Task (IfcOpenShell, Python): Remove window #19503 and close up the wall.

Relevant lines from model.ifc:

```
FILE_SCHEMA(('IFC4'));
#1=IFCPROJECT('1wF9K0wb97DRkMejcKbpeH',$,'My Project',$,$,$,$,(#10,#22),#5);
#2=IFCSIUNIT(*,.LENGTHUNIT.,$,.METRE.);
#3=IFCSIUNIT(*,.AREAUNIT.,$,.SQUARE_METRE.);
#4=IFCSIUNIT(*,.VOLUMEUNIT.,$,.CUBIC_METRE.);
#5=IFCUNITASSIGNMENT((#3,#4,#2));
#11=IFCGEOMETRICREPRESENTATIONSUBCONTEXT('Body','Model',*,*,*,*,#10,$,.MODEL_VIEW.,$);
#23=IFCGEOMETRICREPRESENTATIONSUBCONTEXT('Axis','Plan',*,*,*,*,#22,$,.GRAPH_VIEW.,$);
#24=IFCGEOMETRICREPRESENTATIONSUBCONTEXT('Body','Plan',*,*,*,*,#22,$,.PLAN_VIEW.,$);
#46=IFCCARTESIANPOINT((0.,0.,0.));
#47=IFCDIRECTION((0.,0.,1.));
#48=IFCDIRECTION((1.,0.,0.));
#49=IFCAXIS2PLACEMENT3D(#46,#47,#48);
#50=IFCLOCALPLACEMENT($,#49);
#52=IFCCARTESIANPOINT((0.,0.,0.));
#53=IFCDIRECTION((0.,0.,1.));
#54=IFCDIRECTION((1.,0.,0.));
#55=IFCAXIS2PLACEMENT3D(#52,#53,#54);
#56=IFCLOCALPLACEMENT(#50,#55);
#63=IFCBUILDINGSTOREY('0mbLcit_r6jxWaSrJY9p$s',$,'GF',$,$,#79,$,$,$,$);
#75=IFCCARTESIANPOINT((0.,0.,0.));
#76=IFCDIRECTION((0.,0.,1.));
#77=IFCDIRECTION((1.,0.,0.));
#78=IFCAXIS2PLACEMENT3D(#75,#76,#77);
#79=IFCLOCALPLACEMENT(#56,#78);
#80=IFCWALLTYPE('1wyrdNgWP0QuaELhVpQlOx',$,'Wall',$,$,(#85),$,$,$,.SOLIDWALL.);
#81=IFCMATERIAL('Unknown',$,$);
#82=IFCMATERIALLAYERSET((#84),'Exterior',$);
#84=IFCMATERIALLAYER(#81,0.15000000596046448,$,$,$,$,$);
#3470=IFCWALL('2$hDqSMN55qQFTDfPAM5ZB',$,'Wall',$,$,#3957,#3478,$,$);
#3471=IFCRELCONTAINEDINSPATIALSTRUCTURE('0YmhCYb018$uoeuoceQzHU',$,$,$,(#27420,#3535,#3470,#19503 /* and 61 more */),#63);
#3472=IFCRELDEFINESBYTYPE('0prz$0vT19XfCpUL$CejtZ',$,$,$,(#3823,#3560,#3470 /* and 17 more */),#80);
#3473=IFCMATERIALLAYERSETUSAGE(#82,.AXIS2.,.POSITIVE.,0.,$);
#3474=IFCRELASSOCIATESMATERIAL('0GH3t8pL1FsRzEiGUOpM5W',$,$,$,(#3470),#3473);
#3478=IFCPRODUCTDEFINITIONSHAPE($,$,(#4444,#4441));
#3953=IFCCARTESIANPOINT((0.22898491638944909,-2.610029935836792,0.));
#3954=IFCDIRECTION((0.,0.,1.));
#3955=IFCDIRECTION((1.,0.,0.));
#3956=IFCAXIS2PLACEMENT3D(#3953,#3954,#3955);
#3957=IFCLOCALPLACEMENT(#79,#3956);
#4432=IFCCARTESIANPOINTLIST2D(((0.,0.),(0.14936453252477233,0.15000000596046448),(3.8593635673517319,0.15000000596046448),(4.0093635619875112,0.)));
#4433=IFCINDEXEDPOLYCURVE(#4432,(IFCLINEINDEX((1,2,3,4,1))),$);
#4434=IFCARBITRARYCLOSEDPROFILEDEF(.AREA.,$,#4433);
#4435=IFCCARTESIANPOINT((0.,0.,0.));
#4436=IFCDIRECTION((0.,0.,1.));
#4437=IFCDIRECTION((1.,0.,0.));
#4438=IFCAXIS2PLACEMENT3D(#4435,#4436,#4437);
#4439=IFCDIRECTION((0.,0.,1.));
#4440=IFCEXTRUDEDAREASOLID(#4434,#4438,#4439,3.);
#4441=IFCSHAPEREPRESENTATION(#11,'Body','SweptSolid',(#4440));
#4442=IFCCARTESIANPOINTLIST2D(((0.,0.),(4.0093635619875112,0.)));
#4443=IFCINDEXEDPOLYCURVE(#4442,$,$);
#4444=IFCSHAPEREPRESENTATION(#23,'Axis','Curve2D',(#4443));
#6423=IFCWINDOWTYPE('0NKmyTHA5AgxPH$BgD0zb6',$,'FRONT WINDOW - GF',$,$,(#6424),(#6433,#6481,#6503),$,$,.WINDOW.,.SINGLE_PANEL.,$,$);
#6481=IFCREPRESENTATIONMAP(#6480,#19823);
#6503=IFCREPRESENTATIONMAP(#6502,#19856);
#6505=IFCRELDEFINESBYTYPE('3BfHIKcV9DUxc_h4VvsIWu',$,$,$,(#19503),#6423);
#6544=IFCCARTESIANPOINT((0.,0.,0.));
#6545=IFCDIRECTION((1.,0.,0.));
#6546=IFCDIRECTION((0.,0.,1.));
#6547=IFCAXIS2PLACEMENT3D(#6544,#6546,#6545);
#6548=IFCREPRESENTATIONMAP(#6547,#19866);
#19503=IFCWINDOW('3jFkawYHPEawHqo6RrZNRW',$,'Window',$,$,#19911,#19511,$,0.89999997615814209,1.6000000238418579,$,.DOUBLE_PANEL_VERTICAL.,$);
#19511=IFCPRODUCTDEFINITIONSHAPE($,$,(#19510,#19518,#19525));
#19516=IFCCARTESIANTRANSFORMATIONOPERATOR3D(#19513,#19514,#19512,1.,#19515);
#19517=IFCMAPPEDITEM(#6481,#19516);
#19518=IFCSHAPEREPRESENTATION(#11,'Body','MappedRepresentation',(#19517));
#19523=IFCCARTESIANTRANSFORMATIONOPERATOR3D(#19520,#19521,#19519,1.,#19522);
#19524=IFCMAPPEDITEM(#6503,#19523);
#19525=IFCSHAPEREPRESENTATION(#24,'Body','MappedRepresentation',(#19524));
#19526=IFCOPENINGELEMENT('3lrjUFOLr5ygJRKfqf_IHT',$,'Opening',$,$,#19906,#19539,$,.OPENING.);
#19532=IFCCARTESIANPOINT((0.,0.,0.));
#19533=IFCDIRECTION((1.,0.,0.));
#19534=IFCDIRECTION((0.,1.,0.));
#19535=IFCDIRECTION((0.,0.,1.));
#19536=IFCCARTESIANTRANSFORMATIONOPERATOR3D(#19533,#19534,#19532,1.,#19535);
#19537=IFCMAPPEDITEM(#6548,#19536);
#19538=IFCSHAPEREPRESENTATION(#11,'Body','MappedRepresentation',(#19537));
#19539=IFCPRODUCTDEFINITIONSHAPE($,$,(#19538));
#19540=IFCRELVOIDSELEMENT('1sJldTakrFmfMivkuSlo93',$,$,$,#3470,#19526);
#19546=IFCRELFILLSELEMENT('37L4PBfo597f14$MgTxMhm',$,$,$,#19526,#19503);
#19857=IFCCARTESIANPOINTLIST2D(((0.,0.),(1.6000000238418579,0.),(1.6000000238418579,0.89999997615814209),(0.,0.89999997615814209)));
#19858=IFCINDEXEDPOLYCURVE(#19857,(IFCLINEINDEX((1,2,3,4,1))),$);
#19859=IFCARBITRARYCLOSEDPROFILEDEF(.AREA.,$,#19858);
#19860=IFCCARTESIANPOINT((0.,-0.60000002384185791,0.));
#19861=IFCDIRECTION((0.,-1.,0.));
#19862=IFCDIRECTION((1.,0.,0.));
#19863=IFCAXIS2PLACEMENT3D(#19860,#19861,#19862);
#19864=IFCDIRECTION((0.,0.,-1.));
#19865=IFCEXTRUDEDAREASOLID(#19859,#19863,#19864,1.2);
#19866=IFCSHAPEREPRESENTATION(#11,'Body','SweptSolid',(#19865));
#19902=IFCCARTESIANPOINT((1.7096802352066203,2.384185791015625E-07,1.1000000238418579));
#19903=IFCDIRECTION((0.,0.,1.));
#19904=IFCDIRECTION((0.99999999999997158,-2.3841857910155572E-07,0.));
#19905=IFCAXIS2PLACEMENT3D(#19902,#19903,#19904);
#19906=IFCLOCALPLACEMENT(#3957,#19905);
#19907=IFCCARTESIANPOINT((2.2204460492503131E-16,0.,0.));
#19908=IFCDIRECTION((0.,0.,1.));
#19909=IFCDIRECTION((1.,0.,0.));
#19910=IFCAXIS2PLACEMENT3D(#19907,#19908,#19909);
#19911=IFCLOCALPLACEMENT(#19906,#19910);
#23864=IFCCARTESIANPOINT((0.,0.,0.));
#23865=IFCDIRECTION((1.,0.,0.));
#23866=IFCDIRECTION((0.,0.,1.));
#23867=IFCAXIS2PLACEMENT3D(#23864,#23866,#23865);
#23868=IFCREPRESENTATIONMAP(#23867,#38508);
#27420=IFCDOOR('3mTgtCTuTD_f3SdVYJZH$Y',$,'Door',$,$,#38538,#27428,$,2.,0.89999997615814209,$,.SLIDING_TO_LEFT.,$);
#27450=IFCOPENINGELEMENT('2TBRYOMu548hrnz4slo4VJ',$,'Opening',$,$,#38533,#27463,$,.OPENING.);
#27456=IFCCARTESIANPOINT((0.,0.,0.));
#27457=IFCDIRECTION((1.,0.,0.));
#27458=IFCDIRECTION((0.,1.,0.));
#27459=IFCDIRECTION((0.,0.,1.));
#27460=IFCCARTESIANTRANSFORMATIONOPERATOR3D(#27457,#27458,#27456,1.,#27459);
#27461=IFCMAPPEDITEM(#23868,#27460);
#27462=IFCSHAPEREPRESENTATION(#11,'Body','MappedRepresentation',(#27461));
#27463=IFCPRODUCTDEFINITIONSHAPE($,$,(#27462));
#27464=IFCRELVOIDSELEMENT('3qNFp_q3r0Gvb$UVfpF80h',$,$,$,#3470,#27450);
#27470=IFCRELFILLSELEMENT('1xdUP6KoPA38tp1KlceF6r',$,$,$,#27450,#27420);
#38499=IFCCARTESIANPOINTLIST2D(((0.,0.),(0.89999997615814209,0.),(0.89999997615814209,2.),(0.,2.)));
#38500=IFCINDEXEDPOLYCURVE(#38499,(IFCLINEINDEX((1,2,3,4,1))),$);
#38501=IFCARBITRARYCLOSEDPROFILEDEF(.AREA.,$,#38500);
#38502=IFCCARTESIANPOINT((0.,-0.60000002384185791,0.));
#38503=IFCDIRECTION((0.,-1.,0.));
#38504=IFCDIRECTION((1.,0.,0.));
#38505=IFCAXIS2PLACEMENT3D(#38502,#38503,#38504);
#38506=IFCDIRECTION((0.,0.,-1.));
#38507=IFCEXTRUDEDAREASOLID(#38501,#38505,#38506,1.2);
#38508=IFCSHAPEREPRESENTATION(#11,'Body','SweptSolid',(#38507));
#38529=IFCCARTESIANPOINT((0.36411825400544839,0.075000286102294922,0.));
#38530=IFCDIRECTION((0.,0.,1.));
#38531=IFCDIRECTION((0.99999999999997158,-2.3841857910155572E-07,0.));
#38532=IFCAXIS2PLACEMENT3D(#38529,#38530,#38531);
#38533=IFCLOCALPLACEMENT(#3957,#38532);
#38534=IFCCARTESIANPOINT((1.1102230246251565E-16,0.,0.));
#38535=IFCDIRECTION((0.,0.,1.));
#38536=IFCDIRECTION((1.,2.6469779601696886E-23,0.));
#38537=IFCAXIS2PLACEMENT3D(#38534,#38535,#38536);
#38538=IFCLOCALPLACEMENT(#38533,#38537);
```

```python
import ifcopenshell
import ifcopenshell.api.feature
import ifcopenshell.api.root
import ifcopenshell.geom
import ifcopenshell.util.shape

model = ifcopenshell.open("model.ifc")
settings = ifcopenshell.geom.settings()


def volume(element):
    """Net volume in cubic metres, openings subtracted."""
    shape = ifcopenshell.geom.create_shape(settings, element)
    return ifcopenshell.util.shape.get_volume(shape.geometry)


window = model.by_id(19503)
opening = window.FillsVoids[0].RelatingOpeningElement
wall = opening.VoidsElements[0].RelatingBuildingElement
before = volume(wall)

ifcopenshell.api.root.remove_product(model, product=window)
ifcopenshell.api.feature.remove_feature(model, feature=opening)

after = volume(wall)

print(f"wall volume {before:.3f} -> {after:.3f} m3")

model.write("model_edited.ifc")
```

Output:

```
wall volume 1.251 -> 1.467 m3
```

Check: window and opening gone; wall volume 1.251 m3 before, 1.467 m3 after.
